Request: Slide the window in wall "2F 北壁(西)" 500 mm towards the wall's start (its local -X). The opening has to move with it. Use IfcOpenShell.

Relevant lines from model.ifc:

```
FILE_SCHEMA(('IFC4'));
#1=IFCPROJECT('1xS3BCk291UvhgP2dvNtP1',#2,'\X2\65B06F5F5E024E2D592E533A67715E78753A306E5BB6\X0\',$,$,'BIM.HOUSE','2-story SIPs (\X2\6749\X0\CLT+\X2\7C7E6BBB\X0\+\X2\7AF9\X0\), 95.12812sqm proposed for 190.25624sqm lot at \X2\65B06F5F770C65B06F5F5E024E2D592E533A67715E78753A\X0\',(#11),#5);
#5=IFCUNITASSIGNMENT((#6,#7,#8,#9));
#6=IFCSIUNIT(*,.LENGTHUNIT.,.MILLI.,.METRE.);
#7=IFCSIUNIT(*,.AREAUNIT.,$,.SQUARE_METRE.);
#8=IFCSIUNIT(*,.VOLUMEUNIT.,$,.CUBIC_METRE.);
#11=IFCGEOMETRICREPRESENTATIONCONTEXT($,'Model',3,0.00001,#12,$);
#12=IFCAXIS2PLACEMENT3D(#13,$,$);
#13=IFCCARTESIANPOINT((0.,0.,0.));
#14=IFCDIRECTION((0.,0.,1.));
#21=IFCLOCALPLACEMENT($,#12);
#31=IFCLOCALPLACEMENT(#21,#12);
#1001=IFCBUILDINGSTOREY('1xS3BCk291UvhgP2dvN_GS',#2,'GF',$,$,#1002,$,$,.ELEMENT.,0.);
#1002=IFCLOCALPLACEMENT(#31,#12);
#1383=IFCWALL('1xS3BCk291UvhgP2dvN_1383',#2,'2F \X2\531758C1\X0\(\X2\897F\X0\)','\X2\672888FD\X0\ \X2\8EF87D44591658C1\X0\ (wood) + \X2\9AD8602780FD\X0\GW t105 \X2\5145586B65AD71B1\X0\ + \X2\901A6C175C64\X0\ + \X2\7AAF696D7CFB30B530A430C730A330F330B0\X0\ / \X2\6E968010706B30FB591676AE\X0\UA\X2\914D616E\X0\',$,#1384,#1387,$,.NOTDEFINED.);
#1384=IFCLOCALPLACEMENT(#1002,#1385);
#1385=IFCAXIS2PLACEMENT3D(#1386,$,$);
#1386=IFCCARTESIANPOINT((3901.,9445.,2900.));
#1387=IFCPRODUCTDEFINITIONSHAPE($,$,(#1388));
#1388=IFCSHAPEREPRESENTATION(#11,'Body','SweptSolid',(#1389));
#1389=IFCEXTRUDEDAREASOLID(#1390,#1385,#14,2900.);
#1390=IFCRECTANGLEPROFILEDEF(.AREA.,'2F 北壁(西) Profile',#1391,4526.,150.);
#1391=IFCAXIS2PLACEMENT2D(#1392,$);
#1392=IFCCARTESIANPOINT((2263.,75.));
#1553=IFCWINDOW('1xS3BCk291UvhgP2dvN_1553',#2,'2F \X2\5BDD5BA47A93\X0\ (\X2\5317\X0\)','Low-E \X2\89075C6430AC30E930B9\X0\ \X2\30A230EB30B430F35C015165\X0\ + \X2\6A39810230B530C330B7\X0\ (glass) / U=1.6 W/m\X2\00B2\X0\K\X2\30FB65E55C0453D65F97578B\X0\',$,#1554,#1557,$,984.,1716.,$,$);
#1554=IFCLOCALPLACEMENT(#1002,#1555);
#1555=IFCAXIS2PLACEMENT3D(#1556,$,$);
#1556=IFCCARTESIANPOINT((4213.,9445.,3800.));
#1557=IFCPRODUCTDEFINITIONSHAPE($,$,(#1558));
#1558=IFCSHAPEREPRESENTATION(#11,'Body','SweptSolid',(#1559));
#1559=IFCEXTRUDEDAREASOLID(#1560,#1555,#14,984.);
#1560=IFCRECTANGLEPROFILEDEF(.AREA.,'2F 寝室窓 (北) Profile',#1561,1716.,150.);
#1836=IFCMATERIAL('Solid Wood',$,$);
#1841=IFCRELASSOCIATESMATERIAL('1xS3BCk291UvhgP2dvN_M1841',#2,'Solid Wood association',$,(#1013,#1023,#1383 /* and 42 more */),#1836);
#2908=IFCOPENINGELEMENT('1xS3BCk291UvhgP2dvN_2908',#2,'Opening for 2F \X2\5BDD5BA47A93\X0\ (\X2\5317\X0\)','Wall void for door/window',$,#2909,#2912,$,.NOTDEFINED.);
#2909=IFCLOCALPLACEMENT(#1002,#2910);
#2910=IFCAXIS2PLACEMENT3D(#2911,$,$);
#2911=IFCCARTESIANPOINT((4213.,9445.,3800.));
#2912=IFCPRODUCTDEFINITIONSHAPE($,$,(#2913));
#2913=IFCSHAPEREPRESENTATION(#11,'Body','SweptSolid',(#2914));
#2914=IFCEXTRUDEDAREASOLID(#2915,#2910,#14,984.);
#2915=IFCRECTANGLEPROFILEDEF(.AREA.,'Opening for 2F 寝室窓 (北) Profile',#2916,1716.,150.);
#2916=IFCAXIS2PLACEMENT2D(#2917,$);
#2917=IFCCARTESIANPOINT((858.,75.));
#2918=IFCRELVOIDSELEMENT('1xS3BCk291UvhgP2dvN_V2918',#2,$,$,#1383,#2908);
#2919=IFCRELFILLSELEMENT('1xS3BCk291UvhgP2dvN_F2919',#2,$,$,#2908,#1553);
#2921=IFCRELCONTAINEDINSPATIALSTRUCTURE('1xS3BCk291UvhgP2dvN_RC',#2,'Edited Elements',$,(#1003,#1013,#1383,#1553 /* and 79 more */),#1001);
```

```python
import ifcopenshell
import ifcopenshell.api.geometry
import ifcopenshell.util.placement
import ifcopenshell.util.unit

model = ifcopenshell.open("model.ifc")
unit_scale = ifcopenshell.util.unit.calculate_unit_scale(model)

window = model.by_guid("1xS3BCk291UvhgP2dvN_1553")
opening = window.FillsVoids[0].RelatingOpeningElement
wall = opening.VoidsElements[0].RelatingBuildingElement

wall_matrix = ifcopenshell.util.placement.get_local_placement(wall.ObjectPlacement)
shift = wall_matrix[:3, 0] * -0.5 / unit_scale
before = ifcopenshell.util.placement.get_local_placement(window.ObjectPlacement)[:3, 3].copy()

# The window is not placed relative to its opening, so move both.
for product in (opening, window):
    matrix = ifcopenshell.util.placement.get_local_placement(product.ObjectPlacement)
    matrix[:3, 3] += shift
    ifcopenshell.api.geometry.edit_object_placement(model, product=product, matrix=matrix, is_si=False)

after = ifcopenshell.util.placement.get_local_placement(window.ObjectPlacement)[:3, 3]
print("window moved by", (after - before).round(3) + 0.0)

model.write("model_updated.ifc")
```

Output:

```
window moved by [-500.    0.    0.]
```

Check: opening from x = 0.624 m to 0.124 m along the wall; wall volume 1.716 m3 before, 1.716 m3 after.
